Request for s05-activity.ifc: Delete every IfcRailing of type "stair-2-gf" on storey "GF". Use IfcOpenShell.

First a look at what the model holds.

```python
import ifcopenshell
import ifcopenshell.util.element

model = ifcopenshell.open("s05-activity.ifc")
print(model.schema)
storey = next(s for s in model.by_type("IfcBuildingStorey") if s.Name == "GF")
railings = [e for e in ifcopenshell.util.element.get_decomposition(storey) if e.is_a("IfcRailing")]
seen = {}
for e in railings:
    element_type = ifcopenshell.util.element.get_type(e)
    name = element_type.Name if element_type not in (None, e) else None
    seen[name] = seen.get(name, 0) + 1
for name, count in sorted(seen.items(), key=str):
    print(count, "x", name)
```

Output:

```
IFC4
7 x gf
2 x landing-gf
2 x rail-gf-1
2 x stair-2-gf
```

```python
import ifcopenshell
import ifcopenshell.api.root
import ifcopenshell.util.element

model = ifcopenshell.open("s05-activity.ifc")

storey = next(s for s in model.by_type("IfcBuildingStorey") if s.Name == "GF")
railings = [e for e in ifcopenshell.util.element.get_decomposition(storey) if e.is_a("IfcRailing")]
targets = [e for e in railings if (t := ifcopenshell.util.element.get_type(e)) not in (None, e) and t.Name == "stair-2-gf"]

for e in targets:
    ifcopenshell.api.root.remove_product(model, product=e)
print(len(targets), "removed")

model.write("s05-activity_rev.ifc")
```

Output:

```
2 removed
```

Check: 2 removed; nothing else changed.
